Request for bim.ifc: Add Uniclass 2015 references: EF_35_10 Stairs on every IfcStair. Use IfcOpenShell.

First a look at what the model holds.

```python
import ifcopenshell

model = ifcopenshell.open("bim.ifc")
print(model.schema)
print("classifications:", [c.Name for c in model.by_type("IfcClassification")])
for ifc_class in ("IfcDoor", "IfcRoof", "IfcStair", "IfcWall", "IfcWindow"):
    print(ifc_class, len(model.by_type(ifc_class)))
```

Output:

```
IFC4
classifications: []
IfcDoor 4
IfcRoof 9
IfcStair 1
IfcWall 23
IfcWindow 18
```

```python
import ifcopenshell
import ifcopenshell.api.classification

model = ifcopenshell.open("bim.ifc")

system = ifcopenshell.api.classification.add_classification(model, classification="Uniclass 2015")

codes = {
    "IfcStair": ("EF_35_10", "Stairs"),
}
for ifc_class, (code, name) in codes.items():
    products = model.by_type(ifc_class)
    ifcopenshell.api.classification.add_reference(
        model, products=products, classification=system, identification=code, name=name
    )
    print(code, len(products))

model.write("bim_rev.ifc")
```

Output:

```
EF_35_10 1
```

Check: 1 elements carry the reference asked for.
